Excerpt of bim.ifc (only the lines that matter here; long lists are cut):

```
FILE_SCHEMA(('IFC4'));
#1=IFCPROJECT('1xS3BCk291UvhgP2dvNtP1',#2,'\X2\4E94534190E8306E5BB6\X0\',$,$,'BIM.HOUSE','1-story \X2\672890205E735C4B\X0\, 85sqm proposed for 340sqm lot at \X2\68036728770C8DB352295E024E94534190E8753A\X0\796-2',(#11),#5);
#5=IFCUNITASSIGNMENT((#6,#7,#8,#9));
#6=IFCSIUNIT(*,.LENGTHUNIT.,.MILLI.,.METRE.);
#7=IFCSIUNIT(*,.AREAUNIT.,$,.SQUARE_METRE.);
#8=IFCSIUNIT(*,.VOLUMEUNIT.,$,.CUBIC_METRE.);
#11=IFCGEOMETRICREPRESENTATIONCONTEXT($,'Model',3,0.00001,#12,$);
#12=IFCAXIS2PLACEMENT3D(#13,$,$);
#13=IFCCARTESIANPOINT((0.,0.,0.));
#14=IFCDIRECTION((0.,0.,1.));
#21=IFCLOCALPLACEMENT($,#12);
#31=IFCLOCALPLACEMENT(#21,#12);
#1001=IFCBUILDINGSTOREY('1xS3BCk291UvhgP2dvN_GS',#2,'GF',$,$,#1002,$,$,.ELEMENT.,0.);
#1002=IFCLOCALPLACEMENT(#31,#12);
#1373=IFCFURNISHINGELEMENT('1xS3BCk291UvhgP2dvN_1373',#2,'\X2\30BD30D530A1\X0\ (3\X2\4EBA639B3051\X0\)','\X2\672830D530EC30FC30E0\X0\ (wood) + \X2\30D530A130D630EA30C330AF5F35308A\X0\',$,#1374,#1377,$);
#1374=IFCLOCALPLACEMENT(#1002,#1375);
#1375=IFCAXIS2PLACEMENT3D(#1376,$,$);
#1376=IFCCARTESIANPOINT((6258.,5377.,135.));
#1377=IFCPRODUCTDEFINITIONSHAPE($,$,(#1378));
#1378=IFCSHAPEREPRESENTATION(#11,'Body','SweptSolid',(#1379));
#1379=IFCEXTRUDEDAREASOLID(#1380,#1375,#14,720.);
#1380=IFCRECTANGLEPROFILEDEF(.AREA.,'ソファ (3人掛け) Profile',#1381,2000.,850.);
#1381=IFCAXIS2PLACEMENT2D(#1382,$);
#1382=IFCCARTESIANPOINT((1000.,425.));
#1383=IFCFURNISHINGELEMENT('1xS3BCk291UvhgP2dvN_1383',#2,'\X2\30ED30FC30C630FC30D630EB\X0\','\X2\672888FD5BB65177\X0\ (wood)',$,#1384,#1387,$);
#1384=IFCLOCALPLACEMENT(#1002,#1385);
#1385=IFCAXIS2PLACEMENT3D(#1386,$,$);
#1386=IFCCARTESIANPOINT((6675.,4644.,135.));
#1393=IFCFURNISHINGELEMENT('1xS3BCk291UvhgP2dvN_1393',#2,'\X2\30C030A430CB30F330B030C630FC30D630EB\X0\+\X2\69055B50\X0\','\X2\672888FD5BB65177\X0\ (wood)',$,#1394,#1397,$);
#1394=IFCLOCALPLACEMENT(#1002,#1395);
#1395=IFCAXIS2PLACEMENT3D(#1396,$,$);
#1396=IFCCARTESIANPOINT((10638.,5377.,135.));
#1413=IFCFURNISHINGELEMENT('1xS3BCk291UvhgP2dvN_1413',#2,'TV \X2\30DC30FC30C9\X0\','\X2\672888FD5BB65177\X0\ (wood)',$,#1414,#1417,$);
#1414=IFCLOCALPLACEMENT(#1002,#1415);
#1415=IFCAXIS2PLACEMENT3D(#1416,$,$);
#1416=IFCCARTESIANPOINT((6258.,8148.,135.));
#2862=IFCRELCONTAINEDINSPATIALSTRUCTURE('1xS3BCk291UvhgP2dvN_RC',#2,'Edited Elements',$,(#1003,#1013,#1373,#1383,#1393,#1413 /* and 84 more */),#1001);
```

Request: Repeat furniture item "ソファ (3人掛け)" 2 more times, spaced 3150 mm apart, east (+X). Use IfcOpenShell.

```python
import numpy as np
import ifcopenshell
import ifcopenshell.api.geometry
import ifcopenshell.api.root
import ifcopenshell.util.element
import ifcopenshell.util.placement
import ifcopenshell.util.unit

model = ifcopenshell.open("bim.ifc")
unit_scale = ifcopenshell.util.unit.calculate_unit_scale(model)


def reuse_history(source, copy):
    """copy_class also copies each property set's owner history, people and application; keep the originals."""
    for rel in copy.IsDefinedBy:
        if rel.is_a("IfcRelDefinesByProperties") and (history := rel.RelatingPropertyDefinition.OwnerHistory):
            rel.RelatingPropertyDefinition.OwnerHistory = source.OwnerHistory
            ifcopenshell.util.element.remove_deep2(model, history)


source = model.by_guid("1xS3BCk291UvhgP2dvN_1373")
base = ifcopenshell.util.placement.get_local_placement(source.ObjectPlacement)
step = np.array([1.0, 0.0, 0.0]) * 3.15 / unit_scale

for i in range(1, 3):
    copy = ifcopenshell.api.root.copy_class(model, product=source)
    copy.Representation = ifcopenshell.util.element.copy_deep(
        model, source.Representation, exclude=["IfcGeometricRepresentationContext", "IfcRepresentationMap"]
    )
    reuse_history(source, copy)
    matrix = base.copy()
    matrix[:3, 3] += i * step
    print("added at", matrix[:3, 3].round(3) + 0.0)
    ifcopenshell.api.geometry.edit_object_placement(model, product=copy, matrix=matrix, is_si=False)

model.write("bim_edited.ifc")
```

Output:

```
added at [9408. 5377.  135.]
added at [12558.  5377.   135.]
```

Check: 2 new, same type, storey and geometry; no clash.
